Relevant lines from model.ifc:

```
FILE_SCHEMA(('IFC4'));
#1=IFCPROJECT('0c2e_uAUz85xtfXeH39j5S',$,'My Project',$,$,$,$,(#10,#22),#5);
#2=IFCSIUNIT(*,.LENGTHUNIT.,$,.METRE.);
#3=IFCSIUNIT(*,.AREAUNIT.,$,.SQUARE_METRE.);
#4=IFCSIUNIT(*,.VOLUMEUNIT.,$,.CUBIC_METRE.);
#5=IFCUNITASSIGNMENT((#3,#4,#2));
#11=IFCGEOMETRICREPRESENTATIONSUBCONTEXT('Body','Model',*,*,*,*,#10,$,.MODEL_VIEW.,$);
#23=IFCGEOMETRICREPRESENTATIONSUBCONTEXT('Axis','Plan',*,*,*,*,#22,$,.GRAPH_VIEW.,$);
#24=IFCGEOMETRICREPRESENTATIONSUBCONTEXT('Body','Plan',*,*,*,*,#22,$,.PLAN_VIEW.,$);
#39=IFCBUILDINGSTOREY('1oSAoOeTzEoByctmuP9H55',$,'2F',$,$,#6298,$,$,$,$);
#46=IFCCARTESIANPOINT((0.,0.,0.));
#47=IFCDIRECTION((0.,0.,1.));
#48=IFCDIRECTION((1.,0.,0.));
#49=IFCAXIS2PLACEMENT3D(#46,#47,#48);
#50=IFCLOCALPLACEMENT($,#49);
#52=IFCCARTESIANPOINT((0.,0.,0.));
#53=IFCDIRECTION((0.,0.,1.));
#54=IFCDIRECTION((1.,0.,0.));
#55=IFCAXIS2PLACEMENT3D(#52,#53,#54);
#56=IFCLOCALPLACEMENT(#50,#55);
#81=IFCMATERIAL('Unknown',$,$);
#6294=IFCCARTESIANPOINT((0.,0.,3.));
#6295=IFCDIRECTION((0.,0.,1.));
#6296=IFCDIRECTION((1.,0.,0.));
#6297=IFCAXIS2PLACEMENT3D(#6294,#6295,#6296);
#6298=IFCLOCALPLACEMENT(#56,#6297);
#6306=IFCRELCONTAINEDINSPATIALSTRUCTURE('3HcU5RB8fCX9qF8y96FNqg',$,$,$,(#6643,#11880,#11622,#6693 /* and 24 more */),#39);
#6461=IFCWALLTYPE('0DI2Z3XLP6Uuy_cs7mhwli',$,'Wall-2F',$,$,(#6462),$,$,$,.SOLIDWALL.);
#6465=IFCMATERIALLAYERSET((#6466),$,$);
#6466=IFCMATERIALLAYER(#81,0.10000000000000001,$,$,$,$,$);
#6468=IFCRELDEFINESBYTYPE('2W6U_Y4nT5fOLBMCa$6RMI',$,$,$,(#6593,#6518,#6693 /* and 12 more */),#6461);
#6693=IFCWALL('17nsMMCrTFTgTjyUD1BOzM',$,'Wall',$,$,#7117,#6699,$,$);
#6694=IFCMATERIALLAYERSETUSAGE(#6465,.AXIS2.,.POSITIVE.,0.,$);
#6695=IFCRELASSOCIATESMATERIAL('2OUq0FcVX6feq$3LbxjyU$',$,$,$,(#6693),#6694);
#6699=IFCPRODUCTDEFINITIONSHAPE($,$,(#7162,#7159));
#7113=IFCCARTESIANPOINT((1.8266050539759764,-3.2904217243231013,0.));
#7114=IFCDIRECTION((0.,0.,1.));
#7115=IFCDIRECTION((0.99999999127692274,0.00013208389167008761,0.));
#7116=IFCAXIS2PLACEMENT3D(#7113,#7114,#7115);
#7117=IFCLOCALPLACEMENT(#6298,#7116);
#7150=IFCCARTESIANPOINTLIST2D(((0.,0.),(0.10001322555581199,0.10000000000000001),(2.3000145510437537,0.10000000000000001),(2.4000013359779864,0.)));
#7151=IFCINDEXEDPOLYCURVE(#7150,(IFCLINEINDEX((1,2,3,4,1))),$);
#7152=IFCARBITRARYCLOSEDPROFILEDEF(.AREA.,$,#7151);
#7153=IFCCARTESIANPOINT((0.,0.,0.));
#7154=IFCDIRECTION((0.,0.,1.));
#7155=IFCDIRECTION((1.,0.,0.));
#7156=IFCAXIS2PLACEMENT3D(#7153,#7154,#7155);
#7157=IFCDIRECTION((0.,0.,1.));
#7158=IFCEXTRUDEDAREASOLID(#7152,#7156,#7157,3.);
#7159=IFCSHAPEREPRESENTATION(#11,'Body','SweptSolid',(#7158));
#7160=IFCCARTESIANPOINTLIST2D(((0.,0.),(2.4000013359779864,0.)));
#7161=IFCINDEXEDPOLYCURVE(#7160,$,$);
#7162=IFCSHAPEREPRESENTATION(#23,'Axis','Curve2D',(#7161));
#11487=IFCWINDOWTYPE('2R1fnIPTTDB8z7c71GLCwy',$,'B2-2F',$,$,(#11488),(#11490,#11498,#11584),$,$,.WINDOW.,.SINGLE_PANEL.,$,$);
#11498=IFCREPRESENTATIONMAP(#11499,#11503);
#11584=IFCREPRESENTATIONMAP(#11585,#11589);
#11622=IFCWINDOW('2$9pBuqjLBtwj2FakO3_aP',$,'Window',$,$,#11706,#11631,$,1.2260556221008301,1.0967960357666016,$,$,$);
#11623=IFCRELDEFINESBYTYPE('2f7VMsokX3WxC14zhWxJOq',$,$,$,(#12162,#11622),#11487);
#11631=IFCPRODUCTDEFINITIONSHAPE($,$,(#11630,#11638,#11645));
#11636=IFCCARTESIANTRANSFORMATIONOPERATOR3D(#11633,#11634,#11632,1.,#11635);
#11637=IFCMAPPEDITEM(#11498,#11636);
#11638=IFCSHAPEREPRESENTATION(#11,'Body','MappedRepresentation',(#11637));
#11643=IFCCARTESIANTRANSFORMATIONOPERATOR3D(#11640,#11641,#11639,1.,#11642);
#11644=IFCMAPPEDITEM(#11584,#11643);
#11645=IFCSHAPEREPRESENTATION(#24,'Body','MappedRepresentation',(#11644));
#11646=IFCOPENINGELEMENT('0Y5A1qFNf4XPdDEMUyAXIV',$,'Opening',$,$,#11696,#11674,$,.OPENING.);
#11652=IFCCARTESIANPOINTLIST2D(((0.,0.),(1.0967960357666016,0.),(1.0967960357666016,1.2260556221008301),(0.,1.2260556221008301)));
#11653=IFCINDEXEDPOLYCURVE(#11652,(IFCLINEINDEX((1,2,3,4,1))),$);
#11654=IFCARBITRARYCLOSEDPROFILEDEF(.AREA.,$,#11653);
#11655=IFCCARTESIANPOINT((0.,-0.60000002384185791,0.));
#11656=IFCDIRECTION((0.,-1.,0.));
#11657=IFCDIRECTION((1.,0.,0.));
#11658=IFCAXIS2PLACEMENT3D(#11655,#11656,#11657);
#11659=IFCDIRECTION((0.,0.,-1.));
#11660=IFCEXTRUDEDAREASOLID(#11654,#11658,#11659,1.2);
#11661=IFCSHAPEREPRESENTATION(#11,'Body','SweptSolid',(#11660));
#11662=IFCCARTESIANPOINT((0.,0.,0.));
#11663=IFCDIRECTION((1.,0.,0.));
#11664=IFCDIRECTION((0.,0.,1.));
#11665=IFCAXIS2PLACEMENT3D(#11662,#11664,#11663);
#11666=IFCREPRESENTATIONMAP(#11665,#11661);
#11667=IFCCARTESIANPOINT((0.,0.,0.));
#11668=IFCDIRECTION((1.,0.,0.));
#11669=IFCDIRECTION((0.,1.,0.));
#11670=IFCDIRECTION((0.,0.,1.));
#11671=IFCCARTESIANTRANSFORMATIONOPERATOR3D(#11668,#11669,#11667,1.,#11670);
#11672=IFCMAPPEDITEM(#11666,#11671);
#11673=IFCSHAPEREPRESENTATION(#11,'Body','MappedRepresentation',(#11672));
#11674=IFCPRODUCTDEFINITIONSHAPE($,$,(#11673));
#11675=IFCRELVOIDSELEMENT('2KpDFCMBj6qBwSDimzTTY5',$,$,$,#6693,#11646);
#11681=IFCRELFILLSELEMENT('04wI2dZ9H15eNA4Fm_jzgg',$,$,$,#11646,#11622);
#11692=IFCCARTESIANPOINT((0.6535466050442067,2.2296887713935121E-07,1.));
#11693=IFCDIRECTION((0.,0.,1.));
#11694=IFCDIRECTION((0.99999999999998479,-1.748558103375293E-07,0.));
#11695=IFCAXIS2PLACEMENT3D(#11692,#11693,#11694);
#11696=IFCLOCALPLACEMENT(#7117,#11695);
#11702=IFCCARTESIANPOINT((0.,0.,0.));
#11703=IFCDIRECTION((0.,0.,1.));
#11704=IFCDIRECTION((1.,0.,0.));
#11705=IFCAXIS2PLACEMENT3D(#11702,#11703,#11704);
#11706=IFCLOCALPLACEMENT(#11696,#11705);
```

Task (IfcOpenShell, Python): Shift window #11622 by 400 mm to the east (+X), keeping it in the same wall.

```python
import ifcopenshell
import ifcopenshell.api.geometry
import ifcopenshell.util.placement
import ifcopenshell.util.unit

model = ifcopenshell.open("model.ifc")
unit_scale = ifcopenshell.util.unit.calculate_unit_scale(model)

window = model.by_guid("2$9pBuqjLBtwj2FakO3_aP")
opening = window.FillsVoids[0].RelatingOpeningElement
wall = opening.VoidsElements[0].RelatingBuildingElement

wall_matrix = ifcopenshell.util.placement.get_local_placement(wall.ObjectPlacement)
shift = wall_matrix[:3, 0] * 0.4 / unit_scale
before = ifcopenshell.util.placement.get_local_placement(window.ObjectPlacement)[:3, 3].copy()

# The window is placed relative to its opening, so it follows when the opening moves.
matrix = ifcopenshell.util.placement.get_local_placement(opening.ObjectPlacement)
matrix[:3, 3] += shift
ifcopenshell.api.geometry.edit_object_placement(
    model, product=opening, matrix=matrix, is_si=False, should_transform_children=True
)

after = ifcopenshell.util.placement.get_local_placement(window.ObjectPlacement)[:3, 3]
print("window moved by", (after - before).round(3) + 0.0)

model.write("model-out.ifc")
```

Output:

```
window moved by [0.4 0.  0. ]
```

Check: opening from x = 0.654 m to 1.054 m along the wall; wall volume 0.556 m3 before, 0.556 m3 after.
